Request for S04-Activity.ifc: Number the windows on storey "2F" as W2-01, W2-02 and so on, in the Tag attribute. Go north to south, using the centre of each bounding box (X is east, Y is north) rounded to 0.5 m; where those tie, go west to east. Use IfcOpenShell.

First a look at what the model holds.

```python
import ifcopenshell
import ifcopenshell.util.element
import ifcopenshell.util.placement

model = ifcopenshell.open("S04-Activity.ifc")
print(model.schema)
storey = next(s for s in model.by_type("IfcBuildingStorey") if s.Name == "2F")
windows = [e for e in ifcopenshell.util.element.get_decomposition(storey) if e.is_a("IfcWindow")]
for e in sorted(windows, key=lambda e: e.id()):
    origin = ifcopenshell.util.placement.get_local_placement(e.ObjectPlacement)[:3, 3]
    print(e.id(), e.Tag, e.Name, origin.round(2) + 0.0, sep=" | ")
```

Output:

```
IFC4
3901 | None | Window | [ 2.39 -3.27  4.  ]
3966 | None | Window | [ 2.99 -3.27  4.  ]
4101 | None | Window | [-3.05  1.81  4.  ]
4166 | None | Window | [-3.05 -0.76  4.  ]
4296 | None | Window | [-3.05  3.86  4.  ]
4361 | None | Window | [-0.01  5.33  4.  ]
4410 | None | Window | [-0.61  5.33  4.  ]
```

```python
import ifcopenshell
import ifcopenshell.geom
import ifcopenshell.util.element
import ifcopenshell.util.shape

model = ifcopenshell.open("S04-Activity.ifc")
settings = ifcopenshell.geom.settings()
settings.set("use-world-coords", True)


def centre(element):
    shape = ifcopenshell.geom.create_shape(settings, element)
    return ifcopenshell.util.shape.get_bbox_centroid(shape.geometry)


storey = next(s for s in model.by_type("IfcBuildingStorey") if s.Name == "2F")
windows = [e for e in ifcopenshell.util.element.get_decomposition(storey) if e.is_a("IfcWindow")]

# Insertion points can sit at a corner or the storey origin, so sort by the geometry (in metres).
centres = {e: centre(e) for e in windows}
windows.sort(key=lambda e: (-round(centres[e][1] / 0.5), centres[e][0]))

for i, e in enumerate(windows, start=1):
    number = f"W2-{i:02d}"
    e.Tag = number
    print(e.id(), number)

model.write("S04-Activity_edited.ifc")
```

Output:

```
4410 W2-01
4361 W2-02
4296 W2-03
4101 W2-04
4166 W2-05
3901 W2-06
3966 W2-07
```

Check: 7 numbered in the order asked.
